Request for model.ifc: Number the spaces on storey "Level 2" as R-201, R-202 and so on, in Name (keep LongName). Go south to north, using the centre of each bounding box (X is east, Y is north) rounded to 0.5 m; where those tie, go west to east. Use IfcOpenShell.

First a look at what the model holds.

```python
import ifcopenshell
import ifcopenshell.util.element
import ifcopenshell.util.placement

model = ifcopenshell.open("model.ifc")
print(model.schema)
storey = next(s for s in model.by_type("IfcBuildingStorey") if s.Name == "Level 2")
spaces = [e for e in ifcopenshell.util.element.get_decomposition(storey) if e.is_a("IfcSpace")]
for e in sorted(spaces, key=lambda e: e.id()):
    origin = ifcopenshell.util.placement.get_local_placement(e.ObjectPlacement)[:3, 3]
    print(e.id(), e.Name, e.LongName, origin.round(2) + 0.0, sep=" | ")
```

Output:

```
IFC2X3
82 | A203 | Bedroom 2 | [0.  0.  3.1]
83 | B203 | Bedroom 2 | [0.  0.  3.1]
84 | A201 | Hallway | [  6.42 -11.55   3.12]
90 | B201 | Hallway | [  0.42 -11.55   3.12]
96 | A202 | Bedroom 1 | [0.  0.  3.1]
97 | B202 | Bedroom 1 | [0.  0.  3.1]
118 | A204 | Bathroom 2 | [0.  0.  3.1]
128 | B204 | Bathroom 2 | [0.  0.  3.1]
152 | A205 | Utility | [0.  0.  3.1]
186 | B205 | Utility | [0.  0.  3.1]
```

```python
import ifcopenshell
import ifcopenshell.geom
import ifcopenshell.util.element
import ifcopenshell.util.shape

model = ifcopenshell.open("model.ifc")
settings = ifcopenshell.geom.settings()
settings.set("use-world-coords", True)


def centre(element):
    shape = ifcopenshell.geom.create_shape(settings, element)
    return ifcopenshell.util.shape.get_bbox_centroid(shape.geometry)


storey = next(s for s in model.by_type("IfcBuildingStorey") if s.Name == "Level 2")
spaces = [e for e in ifcopenshell.util.element.get_decomposition(storey) if e.is_a("IfcSpace")]

# Insertion points can sit at a corner or the storey origin, so sort by the geometry (in metres).
centres = {e: centre(e) for e in spaces}
spaces.sort(key=lambda e: (round(centres[e][1] / 0.5), centres[e][0]))

for i, e in enumerate(spaces, start=1):
    number = f"R-2{i:02d}"
    e.Name = number
    print(e.id(), number)

model.write("model_rev.ifc")
```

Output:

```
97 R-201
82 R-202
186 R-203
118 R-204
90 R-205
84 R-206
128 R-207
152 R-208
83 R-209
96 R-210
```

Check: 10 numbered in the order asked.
